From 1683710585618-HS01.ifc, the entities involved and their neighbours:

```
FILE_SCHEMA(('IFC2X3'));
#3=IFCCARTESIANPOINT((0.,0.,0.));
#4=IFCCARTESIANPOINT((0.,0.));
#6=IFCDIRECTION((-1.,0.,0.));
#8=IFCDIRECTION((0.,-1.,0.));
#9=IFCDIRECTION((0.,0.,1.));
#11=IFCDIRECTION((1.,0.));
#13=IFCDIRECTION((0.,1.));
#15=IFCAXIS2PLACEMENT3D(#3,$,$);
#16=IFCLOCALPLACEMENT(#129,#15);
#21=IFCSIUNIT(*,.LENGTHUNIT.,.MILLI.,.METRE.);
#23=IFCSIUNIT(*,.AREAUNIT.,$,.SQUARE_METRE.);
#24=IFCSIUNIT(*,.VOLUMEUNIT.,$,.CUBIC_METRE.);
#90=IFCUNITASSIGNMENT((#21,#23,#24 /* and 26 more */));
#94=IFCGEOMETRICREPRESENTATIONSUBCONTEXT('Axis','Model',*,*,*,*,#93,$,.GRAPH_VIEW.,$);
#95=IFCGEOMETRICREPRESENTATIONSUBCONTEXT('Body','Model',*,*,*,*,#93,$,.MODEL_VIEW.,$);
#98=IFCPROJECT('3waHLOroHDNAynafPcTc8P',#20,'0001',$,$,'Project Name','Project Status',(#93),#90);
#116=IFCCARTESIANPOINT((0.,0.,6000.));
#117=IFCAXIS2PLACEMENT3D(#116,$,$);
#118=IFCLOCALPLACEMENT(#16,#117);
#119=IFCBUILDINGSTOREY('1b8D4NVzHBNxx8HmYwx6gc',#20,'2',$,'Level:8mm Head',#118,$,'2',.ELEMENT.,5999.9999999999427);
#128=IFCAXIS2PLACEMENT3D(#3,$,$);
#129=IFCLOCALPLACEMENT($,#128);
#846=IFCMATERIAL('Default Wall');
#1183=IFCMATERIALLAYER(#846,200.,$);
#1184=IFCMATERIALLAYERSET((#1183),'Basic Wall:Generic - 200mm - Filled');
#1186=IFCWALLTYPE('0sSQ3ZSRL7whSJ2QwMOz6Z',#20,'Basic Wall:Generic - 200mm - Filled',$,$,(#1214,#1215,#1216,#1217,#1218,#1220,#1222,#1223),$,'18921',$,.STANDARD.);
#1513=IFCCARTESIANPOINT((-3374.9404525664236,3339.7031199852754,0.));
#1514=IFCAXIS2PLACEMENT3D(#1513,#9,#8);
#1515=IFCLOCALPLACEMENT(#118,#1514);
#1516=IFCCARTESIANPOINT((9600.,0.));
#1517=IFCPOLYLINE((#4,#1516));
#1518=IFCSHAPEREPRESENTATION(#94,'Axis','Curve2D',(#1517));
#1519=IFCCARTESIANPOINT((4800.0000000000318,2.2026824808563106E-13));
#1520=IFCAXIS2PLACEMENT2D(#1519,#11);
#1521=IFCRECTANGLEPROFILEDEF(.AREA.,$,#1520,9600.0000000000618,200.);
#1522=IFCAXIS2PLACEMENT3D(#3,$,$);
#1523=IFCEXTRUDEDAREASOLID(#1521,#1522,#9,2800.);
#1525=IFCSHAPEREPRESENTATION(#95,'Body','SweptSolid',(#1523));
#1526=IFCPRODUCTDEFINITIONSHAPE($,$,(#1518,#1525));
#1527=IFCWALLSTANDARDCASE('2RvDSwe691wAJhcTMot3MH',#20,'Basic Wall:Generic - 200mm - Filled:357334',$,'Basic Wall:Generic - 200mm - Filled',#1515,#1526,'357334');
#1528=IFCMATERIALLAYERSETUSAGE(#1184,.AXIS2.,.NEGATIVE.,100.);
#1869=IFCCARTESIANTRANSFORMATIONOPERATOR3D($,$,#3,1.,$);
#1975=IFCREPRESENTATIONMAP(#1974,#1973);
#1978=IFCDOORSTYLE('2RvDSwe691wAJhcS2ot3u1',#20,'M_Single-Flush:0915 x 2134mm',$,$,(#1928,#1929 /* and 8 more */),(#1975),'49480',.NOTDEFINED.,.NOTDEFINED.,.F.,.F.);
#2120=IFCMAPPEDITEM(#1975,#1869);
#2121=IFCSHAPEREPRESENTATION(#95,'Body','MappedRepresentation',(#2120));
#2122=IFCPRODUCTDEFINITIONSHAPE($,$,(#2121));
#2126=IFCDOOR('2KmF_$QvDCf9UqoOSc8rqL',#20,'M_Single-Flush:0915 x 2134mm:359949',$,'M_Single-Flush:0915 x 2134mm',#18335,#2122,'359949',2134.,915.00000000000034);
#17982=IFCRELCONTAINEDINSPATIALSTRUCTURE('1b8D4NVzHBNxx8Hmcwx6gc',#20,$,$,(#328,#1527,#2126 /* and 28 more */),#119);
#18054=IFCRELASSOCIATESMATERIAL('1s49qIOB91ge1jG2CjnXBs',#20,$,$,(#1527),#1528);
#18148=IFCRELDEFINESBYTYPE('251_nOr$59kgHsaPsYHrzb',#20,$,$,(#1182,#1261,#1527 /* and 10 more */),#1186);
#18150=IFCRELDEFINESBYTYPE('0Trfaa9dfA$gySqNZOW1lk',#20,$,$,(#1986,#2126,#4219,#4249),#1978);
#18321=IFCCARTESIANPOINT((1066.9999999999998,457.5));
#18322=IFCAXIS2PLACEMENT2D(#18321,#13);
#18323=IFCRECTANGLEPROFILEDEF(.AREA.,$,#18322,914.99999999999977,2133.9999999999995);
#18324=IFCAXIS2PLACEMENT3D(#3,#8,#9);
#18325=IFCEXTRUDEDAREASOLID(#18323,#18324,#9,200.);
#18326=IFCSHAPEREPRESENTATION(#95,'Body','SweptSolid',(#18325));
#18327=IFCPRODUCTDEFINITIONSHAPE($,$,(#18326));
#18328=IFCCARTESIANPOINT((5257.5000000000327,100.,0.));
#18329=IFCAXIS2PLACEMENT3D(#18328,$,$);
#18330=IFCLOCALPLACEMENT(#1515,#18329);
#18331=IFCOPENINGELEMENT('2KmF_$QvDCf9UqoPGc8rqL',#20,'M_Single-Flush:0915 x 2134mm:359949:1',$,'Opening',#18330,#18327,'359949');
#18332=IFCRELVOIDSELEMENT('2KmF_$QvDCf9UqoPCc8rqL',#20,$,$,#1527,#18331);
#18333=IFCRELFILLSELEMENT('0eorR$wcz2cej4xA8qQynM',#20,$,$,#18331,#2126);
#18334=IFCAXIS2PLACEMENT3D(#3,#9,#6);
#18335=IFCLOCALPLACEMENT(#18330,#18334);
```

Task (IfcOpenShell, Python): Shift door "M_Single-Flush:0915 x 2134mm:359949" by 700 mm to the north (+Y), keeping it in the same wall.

```python
import ifcopenshell
import ifcopenshell.api.geometry
import ifcopenshell.util.placement

model = ifcopenshell.open("1683710585618-HS01.ifc")

door = model.by_id(2126)
opening = door.FillsVoids[0].RelatingOpeningElement
wall = opening.VoidsElements[0].RelatingBuildingElement

wall_matrix = ifcopenshell.util.placement.get_local_placement(wall.ObjectPlacement)
shift = wall_matrix[:3, 0] * -700.0
before = ifcopenshell.util.placement.get_local_placement(door.ObjectPlacement)[:3, 3].copy()

# The door is placed relative to its opening, so it follows when the opening moves.
matrix = ifcopenshell.util.placement.get_local_placement(opening.ObjectPlacement)
matrix[:3, 3] += shift
ifcopenshell.api.geometry.edit_object_placement(
    model, product=opening, matrix=matrix, is_si=False, should_transform_children=True
)

after = ifcopenshell.util.placement.get_local_placement(door.ObjectPlacement)[:3, 3]
print("door moved by", (after - before).round(3) + 0.0)

model.write("1683710585618-HS01_v2.ifc")
```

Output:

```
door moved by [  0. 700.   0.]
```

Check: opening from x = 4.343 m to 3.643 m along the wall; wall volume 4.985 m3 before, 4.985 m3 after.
